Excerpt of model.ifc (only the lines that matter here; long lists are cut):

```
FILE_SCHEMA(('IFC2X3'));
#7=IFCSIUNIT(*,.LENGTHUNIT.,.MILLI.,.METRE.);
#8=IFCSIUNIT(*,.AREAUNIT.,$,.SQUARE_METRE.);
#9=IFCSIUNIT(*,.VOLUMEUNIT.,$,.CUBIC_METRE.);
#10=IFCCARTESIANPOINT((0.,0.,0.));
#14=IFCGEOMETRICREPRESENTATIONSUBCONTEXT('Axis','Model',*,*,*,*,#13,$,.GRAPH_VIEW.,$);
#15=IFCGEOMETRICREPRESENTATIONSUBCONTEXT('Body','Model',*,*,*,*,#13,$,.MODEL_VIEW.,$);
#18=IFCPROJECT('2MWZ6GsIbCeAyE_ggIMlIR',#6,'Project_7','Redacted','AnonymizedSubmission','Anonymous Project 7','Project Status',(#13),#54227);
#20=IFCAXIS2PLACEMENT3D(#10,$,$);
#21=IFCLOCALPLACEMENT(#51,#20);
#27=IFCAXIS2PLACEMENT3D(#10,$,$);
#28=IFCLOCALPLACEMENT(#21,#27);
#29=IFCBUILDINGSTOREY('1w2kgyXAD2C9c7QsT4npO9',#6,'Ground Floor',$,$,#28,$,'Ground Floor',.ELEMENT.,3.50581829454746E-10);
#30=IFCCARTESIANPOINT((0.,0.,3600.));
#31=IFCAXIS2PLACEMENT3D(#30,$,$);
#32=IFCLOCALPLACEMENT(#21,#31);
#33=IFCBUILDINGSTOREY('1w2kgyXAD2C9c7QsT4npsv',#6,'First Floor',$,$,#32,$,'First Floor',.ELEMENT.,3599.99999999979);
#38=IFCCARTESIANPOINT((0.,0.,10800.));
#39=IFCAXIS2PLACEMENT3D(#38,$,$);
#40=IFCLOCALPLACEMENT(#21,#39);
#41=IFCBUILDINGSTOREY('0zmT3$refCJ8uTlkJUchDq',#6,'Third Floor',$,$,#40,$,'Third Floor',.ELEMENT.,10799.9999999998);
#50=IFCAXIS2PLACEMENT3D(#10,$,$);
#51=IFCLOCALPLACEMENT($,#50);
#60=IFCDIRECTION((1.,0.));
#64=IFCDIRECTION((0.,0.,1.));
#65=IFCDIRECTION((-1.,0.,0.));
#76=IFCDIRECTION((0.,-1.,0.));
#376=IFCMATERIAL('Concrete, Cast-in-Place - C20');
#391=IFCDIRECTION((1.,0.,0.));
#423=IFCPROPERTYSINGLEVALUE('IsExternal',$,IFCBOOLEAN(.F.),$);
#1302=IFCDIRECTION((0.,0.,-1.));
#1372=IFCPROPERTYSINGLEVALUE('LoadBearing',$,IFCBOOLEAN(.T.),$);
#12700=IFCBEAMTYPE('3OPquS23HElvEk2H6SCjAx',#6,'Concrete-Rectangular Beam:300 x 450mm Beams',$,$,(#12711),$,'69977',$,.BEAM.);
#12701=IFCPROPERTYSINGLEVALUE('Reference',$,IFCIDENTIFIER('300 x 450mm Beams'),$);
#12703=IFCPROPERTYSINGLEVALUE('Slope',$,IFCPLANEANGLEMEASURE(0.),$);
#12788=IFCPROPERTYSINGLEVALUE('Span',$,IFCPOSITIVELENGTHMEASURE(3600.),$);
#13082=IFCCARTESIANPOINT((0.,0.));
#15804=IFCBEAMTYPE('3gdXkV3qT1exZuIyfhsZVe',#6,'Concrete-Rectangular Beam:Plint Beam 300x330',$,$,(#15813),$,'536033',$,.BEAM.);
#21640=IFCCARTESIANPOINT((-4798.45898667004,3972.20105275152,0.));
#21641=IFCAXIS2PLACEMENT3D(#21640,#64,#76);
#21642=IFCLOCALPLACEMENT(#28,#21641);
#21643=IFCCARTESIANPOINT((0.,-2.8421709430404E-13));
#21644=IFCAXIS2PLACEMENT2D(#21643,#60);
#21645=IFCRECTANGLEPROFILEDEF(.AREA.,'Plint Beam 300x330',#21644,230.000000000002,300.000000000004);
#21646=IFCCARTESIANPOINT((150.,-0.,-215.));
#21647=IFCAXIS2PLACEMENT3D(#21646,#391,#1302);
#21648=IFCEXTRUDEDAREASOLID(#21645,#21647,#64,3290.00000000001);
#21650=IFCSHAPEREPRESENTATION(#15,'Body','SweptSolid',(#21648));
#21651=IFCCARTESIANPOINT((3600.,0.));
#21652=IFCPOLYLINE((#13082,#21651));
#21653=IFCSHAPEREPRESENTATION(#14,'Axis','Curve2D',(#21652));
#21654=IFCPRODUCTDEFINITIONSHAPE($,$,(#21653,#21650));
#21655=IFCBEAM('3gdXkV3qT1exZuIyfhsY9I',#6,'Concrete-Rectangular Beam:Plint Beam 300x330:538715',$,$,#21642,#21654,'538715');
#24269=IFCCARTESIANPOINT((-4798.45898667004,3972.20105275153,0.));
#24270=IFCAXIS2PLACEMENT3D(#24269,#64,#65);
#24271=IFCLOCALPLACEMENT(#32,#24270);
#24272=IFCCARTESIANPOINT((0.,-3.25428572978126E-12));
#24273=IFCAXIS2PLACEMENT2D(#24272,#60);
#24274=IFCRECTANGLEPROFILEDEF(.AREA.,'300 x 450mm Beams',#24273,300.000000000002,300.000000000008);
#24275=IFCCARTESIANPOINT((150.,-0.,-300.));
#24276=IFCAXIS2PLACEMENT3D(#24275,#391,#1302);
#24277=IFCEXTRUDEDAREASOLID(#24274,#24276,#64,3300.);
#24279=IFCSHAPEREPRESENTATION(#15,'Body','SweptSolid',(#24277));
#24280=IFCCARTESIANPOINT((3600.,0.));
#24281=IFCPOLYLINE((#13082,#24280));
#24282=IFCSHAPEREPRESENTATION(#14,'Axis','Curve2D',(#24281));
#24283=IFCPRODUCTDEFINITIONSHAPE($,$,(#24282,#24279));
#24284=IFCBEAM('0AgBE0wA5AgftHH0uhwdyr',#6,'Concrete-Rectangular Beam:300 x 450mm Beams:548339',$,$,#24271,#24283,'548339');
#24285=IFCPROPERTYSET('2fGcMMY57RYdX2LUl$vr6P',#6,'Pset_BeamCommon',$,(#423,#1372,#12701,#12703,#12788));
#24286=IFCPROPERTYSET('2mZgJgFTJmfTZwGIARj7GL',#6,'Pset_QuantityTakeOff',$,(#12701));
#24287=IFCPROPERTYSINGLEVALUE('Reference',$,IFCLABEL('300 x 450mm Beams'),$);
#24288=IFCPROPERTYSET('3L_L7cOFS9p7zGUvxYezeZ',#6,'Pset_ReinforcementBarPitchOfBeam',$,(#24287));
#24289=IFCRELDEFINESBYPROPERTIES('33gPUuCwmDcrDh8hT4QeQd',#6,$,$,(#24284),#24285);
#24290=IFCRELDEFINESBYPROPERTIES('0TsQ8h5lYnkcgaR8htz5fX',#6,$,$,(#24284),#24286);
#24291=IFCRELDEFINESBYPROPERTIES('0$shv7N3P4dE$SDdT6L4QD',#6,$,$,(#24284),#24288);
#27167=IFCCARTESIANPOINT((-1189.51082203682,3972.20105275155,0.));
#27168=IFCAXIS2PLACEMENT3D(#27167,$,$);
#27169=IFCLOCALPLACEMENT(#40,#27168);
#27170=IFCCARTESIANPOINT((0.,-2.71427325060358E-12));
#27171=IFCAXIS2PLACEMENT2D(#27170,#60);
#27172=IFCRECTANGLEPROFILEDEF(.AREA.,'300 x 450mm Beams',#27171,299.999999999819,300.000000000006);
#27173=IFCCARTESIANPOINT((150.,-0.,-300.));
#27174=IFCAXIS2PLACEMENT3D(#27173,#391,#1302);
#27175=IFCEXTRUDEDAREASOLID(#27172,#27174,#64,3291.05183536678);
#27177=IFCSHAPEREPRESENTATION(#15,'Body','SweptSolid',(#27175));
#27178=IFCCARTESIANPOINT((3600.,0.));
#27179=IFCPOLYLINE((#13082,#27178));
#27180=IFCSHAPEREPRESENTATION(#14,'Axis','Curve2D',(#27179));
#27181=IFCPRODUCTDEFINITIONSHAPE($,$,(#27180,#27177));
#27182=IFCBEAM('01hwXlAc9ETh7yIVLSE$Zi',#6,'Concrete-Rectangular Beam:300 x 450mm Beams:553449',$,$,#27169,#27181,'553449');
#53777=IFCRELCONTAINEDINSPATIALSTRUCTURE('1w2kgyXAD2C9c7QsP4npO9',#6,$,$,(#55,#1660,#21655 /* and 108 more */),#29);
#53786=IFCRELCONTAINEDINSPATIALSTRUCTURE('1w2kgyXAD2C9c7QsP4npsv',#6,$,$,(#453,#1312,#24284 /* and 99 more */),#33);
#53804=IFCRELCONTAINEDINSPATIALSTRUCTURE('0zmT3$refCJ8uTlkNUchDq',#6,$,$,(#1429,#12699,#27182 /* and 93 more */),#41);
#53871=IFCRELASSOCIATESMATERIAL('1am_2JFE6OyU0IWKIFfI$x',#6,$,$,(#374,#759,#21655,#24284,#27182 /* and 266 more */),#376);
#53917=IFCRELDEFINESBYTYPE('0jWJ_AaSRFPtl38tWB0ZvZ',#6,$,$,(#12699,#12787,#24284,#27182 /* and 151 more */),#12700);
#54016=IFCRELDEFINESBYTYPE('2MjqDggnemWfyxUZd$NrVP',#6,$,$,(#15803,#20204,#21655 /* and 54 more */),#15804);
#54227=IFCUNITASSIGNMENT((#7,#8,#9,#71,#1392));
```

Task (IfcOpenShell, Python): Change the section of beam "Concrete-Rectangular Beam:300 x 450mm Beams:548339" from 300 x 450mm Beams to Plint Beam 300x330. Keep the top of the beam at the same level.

```python
import ifcopenshell
import ifcopenshell.api.pset
import ifcopenshell.api.type
import ifcopenshell.util.element
import ifcopenshell.util.representation

model = ifcopenshell.open("model.ifc")

member = model.by_id(24284)
source = next(p for p in model.by_type("IfcRectangleProfileDef") if p.ProfileName == "Plint Beam 300x330")

body = ifcopenshell.util.representation.get_representation(member, "Model", "Body")
solid = body.Items[0]
old_profile = solid.SweptArea

# Copy the section's sizes but keep this member's own profile position.
profile = ifcopenshell.util.element.copy(model, source)
# Profiles are centred, so shift by half the change in depth to hold the top.
shift = (old_profile.XDim - profile.XDim) / 2
x, y = old_profile.Position.Location.Coordinates
up = (-1.0, 0.0)  # upwards, in the solid's own plane
location = model.createIfcCartesianPoint((x + up[0] * shift, y + up[1] * shift))
profile.Position = model.createIfcAxis2Placement2D(location, old_profile.Position.RefDirection)
solid.SweptArea = profile
if not model.get_total_inverses(old_profile):
    ifcopenshell.util.element.remove_deep2(model, old_profile)

new_type = model.by_guid("3gdXkV3qT1exZuIyfhsZVe")
ifcopenshell.api.type.assign_type(
    model, related_objects=[member], relating_type=new_type, should_map_representations=False
)
member.Name = member.Name.replace("300 x 450mm Beams", "Plint Beam 300x330")
pset = model.by_id(ifcopenshell.util.element.get_pset(member, "Pset_BeamCommon", should_inherit=False)["id"])
ifcopenshell.api.pset.edit_pset(model, pset=pset, properties={"Reference": "Plint Beam 300x330"})
pset = model.by_id(ifcopenshell.util.element.get_pset(member, "Pset_QuantityTakeOff", should_inherit=False)["id"])
ifcopenshell.api.pset.edit_pset(model, pset=pset, properties={"Reference": "Plint Beam 300x330"})
pset = model.by_id(ifcopenshell.util.element.get_pset(member, "Pset_ReinforcementBarPitchOfBeam", should_inherit=False)["id"])
ifcopenshell.api.pset.edit_pset(model, pset=pset, properties={"Reference": "Plint Beam 300x330"})

print(solid.SweptArea)

model.write("model_rev.ifc")
```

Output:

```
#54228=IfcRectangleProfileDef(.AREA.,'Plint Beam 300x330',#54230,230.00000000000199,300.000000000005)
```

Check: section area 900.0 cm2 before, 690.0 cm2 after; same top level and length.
